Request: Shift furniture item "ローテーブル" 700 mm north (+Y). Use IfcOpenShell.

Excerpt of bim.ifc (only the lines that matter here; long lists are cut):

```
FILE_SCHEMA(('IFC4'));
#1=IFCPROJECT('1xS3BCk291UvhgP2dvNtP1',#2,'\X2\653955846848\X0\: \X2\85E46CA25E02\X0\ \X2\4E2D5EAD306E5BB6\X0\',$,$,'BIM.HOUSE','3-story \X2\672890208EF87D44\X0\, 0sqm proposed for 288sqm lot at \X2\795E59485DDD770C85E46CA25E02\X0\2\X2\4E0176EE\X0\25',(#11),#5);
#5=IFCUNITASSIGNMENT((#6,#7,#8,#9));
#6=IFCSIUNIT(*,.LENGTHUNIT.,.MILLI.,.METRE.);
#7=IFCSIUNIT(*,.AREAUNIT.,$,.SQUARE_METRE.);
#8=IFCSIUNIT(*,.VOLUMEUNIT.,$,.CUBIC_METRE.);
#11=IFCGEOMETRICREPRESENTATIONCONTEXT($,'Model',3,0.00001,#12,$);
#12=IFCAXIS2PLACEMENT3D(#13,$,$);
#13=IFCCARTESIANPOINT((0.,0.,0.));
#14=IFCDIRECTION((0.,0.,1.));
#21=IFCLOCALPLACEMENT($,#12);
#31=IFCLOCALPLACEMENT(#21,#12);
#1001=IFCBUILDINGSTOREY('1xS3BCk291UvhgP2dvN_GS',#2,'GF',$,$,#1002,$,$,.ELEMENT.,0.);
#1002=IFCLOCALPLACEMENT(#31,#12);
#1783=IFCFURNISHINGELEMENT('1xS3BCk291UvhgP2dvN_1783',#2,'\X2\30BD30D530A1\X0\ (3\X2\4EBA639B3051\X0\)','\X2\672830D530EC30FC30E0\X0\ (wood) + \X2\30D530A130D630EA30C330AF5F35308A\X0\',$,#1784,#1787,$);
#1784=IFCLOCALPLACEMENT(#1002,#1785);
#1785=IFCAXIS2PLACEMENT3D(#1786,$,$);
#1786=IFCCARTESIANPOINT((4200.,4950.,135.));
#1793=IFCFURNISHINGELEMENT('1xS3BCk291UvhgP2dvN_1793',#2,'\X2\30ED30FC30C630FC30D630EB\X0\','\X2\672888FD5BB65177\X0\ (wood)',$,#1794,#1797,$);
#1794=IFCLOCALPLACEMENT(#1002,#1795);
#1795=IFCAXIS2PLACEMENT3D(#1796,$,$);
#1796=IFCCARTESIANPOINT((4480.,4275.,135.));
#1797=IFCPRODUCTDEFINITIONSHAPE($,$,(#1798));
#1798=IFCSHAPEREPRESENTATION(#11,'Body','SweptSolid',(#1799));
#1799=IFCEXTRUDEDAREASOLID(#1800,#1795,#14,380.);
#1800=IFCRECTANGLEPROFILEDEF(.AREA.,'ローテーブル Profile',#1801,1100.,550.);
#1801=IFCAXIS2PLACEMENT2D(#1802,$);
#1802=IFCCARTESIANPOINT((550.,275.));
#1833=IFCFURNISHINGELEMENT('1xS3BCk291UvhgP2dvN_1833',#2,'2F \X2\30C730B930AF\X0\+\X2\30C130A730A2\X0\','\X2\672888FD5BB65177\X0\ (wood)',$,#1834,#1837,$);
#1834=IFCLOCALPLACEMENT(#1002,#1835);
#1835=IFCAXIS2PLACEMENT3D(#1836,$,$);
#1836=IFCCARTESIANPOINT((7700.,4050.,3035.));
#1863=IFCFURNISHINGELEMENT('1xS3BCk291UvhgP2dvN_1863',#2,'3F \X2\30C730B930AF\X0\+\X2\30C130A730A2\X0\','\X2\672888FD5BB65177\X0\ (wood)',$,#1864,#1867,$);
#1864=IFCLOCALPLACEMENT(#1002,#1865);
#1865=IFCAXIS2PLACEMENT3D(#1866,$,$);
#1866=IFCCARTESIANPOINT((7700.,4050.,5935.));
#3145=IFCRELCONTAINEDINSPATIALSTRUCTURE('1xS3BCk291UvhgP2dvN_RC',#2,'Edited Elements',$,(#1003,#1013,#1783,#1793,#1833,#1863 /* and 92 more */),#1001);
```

```python
import ifcopenshell
import ifcopenshell.api.geometry
import ifcopenshell.util.placement
import ifcopenshell.util.unit

model = ifcopenshell.open("bim.ifc")
unit_scale = ifcopenshell.util.unit.calculate_unit_scale(model)

item = model.by_id(1793)
matrix = ifcopenshell.util.placement.get_local_placement(item.ObjectPlacement)
matrix[1, 3] += 0.7 / unit_scale
ifcopenshell.api.geometry.edit_object_placement(model, product=item, matrix=matrix, is_si=False)

print(ifcopenshell.util.placement.get_local_placement(item.ObjectPlacement).round(3) + 0.0)

model.write("bim_v2.ifc")
```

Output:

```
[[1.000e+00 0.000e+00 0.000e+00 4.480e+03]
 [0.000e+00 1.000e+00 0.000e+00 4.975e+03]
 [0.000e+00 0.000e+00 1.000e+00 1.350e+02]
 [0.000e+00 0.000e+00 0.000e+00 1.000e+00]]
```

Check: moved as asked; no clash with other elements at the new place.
